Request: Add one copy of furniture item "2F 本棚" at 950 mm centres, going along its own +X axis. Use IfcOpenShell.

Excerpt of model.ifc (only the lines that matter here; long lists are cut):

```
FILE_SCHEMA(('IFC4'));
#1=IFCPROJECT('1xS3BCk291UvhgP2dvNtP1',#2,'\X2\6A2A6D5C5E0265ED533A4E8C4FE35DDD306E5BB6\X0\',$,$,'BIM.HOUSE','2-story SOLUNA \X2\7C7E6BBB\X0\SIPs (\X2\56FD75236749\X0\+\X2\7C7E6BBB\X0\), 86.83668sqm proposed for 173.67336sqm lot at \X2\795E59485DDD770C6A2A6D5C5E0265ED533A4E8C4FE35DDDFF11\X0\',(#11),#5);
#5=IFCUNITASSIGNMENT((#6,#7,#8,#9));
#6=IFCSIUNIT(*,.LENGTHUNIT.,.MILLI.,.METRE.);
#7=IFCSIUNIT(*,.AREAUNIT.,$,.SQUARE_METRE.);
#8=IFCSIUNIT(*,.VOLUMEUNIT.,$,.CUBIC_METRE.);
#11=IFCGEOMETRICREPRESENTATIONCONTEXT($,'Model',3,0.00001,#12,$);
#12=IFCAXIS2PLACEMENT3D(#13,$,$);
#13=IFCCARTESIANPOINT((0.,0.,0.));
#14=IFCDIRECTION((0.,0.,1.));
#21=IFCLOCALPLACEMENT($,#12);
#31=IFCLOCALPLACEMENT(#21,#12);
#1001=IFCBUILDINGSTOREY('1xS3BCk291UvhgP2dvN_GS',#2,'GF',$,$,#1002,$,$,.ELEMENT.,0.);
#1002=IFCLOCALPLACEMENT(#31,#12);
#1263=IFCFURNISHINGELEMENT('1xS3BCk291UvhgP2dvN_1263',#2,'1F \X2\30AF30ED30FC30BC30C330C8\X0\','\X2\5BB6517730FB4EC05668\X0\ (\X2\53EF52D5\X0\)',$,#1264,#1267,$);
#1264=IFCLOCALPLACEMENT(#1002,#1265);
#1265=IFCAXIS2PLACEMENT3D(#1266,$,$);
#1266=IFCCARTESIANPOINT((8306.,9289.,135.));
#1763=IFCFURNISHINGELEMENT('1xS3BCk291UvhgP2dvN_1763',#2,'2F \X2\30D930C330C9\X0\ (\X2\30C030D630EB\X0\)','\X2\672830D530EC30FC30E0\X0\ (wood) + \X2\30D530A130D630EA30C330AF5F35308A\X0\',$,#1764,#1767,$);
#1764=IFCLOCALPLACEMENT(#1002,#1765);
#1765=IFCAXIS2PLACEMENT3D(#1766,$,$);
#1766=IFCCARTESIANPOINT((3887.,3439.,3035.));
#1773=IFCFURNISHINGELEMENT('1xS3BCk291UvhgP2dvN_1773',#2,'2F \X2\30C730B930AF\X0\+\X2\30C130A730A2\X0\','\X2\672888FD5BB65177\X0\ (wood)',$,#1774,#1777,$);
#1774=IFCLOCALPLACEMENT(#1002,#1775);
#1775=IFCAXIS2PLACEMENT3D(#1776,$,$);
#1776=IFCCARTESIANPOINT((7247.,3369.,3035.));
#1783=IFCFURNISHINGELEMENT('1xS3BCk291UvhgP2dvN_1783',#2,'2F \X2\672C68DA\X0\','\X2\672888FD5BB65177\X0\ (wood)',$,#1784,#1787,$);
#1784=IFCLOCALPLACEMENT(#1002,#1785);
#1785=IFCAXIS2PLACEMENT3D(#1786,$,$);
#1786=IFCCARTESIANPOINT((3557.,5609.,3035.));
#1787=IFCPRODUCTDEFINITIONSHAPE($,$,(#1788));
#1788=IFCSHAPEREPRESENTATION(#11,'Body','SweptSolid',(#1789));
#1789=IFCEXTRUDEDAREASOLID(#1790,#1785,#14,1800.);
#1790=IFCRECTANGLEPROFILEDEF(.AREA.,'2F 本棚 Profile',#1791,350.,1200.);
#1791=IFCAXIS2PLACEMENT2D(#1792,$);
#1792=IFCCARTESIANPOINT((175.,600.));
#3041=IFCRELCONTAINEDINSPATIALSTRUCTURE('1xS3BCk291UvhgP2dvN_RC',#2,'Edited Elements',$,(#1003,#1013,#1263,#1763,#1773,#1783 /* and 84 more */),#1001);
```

```python
import ifcopenshell
import ifcopenshell.api.geometry
import ifcopenshell.api.root
import ifcopenshell.util.element
import ifcopenshell.util.placement
import ifcopenshell.util.unit

model = ifcopenshell.open("model.ifc")
unit_scale = ifcopenshell.util.unit.calculate_unit_scale(model)


def reuse_history(source, copy):
    """copy_class also copies each property set's owner history, people and application; keep the originals."""
    for rel in copy.IsDefinedBy:
        if rel.is_a("IfcRelDefinesByProperties") and (history := rel.RelatingPropertyDefinition.OwnerHistory):
            rel.RelatingPropertyDefinition.OwnerHistory = source.OwnerHistory
            ifcopenshell.util.element.remove_deep2(model, history)


source = model.by_guid("1xS3BCk291UvhgP2dvN_1783")
base = ifcopenshell.util.placement.get_local_placement(source.ObjectPlacement)
step = base[:3, 0] * 0.95 / unit_scale

for i in range(1, 2):
    copy = ifcopenshell.api.root.copy_class(model, product=source)
    copy.Representation = ifcopenshell.util.element.copy_deep(
        model, source.Representation, exclude=["IfcGeometricRepresentationContext", "IfcRepresentationMap"]
    )
    reuse_history(source, copy)
    matrix = base.copy()
    matrix[:3, 3] += i * step
    print("added at", matrix[:3, 3].round(3) + 0.0)
    ifcopenshell.api.geometry.edit_object_placement(model, product=copy, matrix=matrix, is_si=False)

model.write("model_v2.ifc")
```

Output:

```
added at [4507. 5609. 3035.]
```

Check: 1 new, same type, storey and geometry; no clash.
